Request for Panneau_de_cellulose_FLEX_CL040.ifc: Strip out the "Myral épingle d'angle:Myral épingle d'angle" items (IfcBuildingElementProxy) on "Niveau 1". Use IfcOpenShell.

First a look at what the model holds.

```python
import ifcopenshell
import ifcopenshell.util.element

model = ifcopenshell.open("Panneau_de_cellulose_FLEX_CL040.ifc")
print(model.schema)
storey = next(s for s in model.by_type("IfcBuildingStorey") if s.Name == "Niveau 1")
proxies = [e for e in ifcopenshell.util.element.get_decomposition(storey) if e.is_a("IfcBuildingElementProxy")]
seen = {}
for e in proxies:
    element_type = ifcopenshell.util.element.get_type(e)
    name = element_type.Name if element_type not in (None, e) else None
    seen[name] = seen.get(name, 0) + 1
for name, count in sorted(seen.items(), key=str):
    print(count, "x", name)
```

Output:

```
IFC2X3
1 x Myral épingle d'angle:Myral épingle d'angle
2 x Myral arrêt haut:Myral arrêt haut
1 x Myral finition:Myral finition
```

```python
import ifcopenshell
import ifcopenshell.api.root
import ifcopenshell.util.element

model = ifcopenshell.open("Panneau_de_cellulose_FLEX_CL040.ifc")

storey = next(s for s in model.by_type("IfcBuildingStorey") if s.Name == "Niveau 1")
proxies = [e for e in ifcopenshell.util.element.get_decomposition(storey) if e.is_a("IfcBuildingElementProxy")]
targets = [e for e in proxies if (t := ifcopenshell.util.element.get_type(e)) not in (None, e) and t.Name == "Myral épingle d'angle:Myral épingle d'angle"]

for e in targets:
    ifcopenshell.api.root.remove_product(model, product=e)
print(len(targets), "removed")

model.write("Panneau_de_cellulose_FLEX_CL040-out.ifc")
```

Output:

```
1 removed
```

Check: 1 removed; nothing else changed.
